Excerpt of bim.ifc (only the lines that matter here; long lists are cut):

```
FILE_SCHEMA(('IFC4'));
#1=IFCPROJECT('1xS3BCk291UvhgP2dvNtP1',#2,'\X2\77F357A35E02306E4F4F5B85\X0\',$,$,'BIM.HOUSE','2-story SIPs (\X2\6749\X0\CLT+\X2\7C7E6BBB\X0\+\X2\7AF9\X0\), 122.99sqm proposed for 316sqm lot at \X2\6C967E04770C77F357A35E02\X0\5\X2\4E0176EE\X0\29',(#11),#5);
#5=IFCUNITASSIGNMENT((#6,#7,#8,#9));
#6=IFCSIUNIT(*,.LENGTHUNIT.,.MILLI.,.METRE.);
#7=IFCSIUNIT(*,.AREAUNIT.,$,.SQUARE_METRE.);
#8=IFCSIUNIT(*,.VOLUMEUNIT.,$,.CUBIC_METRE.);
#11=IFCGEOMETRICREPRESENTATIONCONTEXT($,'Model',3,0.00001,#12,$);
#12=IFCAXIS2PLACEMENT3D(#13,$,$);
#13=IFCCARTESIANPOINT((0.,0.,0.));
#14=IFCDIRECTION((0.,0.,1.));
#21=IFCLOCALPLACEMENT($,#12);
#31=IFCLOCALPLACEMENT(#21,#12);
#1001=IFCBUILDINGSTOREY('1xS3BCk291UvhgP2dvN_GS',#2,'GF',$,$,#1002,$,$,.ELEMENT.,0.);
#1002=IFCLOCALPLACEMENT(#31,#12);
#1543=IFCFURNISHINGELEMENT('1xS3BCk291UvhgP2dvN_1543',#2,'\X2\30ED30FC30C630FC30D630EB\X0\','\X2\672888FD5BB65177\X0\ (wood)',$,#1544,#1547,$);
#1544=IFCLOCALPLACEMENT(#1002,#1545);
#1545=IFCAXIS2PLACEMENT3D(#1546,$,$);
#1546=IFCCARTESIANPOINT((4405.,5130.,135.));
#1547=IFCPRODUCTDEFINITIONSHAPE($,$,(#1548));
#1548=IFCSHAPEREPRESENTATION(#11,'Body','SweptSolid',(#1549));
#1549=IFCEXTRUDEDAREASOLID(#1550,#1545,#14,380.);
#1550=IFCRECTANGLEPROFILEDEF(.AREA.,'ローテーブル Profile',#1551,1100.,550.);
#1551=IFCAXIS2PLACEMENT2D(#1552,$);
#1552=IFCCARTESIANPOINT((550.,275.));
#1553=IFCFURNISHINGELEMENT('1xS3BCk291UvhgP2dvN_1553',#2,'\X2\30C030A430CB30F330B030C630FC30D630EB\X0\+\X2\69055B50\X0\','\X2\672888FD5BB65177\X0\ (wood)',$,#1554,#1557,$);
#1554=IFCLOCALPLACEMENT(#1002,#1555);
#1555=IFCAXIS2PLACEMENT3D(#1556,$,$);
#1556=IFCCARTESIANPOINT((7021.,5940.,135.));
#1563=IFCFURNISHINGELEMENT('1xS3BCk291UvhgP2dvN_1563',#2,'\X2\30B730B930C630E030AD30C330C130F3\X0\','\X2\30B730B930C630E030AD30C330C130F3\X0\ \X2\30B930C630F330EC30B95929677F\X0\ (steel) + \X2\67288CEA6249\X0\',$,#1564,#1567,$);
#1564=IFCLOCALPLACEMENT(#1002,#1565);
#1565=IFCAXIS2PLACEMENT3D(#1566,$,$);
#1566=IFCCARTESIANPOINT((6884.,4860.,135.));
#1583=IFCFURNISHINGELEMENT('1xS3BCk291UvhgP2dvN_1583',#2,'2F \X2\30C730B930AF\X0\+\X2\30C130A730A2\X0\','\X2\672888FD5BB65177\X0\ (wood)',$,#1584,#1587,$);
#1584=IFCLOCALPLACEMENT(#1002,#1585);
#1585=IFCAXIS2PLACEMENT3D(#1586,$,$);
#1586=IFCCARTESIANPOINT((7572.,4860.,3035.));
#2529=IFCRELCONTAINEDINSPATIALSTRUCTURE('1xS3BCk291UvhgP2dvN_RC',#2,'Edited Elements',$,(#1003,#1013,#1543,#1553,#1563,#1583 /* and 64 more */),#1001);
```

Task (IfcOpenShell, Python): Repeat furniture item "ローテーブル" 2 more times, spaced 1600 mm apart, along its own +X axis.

```python
import ifcopenshell
import ifcopenshell.api.geometry
import ifcopenshell.api.root
import ifcopenshell.util.element
import ifcopenshell.util.placement

model = ifcopenshell.open("bim.ifc")


def reuse_history(source, copy):
    """copy_class also copies each property set's owner history, people and application; keep the originals."""
    for rel in copy.IsDefinedBy:
        if rel.is_a("IfcRelDefinesByProperties") and (history := rel.RelatingPropertyDefinition.OwnerHistory):
            rel.RelatingPropertyDefinition.OwnerHistory = source.OwnerHistory
            ifcopenshell.util.element.remove_deep2(model, history)


source = model.by_guid("1xS3BCk291UvhgP2dvN_1543")
base = ifcopenshell.util.placement.get_local_placement(source.ObjectPlacement)
step = base[:3, 0] * 1600.0

for i in range(1, 3):
    copy = ifcopenshell.api.root.copy_class(model, product=source)
    copy.Representation = ifcopenshell.util.element.copy_deep(
        model, source.Representation, exclude=["IfcGeometricRepresentationContext", "IfcRepresentationMap"]
    )
    reuse_history(source, copy)
    matrix = base.copy()
    matrix[:3, 3] += i * step
    print("added at", matrix[:3, 3].round(3) + 0.0)
    ifcopenshell.api.geometry.edit_object_placement(model, product=copy, matrix=matrix, is_si=False)

model.write("bim_edited.ifc")
```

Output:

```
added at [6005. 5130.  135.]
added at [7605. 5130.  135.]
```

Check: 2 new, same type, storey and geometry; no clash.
